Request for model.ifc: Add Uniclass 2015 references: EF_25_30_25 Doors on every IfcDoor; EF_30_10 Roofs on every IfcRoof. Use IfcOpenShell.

First a look at what the model holds.

```python
import ifcopenshell

model = ifcopenshell.open("model.ifc")
print(model.schema)
print("classifications:", [c.Name for c in model.by_type("IfcClassification")])
for ifc_class in ("IfcDoor", "IfcRoof", "IfcStair", "IfcWall", "IfcWindow"):
    print(ifc_class, len(model.by_type(ifc_class)))
```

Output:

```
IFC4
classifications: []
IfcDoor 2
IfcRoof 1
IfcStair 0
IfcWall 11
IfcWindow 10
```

```python
import ifcopenshell
import ifcopenshell.api.classification

model = ifcopenshell.open("model.ifc")

system = ifcopenshell.api.classification.add_classification(model, classification="Uniclass 2015")

codes = {
    "IfcDoor": ("EF_25_30_25", "Doors"),
    "IfcRoof": ("EF_30_10", "Roofs"),
}
for ifc_class, (code, name) in codes.items():
    products = model.by_type(ifc_class)
    ifcopenshell.api.classification.add_reference(
        model, products=products, classification=system, identification=code, name=name
    )
    print(code, len(products))

model.write("model_v2.ifc")
```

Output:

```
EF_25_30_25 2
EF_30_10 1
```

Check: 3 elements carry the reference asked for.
